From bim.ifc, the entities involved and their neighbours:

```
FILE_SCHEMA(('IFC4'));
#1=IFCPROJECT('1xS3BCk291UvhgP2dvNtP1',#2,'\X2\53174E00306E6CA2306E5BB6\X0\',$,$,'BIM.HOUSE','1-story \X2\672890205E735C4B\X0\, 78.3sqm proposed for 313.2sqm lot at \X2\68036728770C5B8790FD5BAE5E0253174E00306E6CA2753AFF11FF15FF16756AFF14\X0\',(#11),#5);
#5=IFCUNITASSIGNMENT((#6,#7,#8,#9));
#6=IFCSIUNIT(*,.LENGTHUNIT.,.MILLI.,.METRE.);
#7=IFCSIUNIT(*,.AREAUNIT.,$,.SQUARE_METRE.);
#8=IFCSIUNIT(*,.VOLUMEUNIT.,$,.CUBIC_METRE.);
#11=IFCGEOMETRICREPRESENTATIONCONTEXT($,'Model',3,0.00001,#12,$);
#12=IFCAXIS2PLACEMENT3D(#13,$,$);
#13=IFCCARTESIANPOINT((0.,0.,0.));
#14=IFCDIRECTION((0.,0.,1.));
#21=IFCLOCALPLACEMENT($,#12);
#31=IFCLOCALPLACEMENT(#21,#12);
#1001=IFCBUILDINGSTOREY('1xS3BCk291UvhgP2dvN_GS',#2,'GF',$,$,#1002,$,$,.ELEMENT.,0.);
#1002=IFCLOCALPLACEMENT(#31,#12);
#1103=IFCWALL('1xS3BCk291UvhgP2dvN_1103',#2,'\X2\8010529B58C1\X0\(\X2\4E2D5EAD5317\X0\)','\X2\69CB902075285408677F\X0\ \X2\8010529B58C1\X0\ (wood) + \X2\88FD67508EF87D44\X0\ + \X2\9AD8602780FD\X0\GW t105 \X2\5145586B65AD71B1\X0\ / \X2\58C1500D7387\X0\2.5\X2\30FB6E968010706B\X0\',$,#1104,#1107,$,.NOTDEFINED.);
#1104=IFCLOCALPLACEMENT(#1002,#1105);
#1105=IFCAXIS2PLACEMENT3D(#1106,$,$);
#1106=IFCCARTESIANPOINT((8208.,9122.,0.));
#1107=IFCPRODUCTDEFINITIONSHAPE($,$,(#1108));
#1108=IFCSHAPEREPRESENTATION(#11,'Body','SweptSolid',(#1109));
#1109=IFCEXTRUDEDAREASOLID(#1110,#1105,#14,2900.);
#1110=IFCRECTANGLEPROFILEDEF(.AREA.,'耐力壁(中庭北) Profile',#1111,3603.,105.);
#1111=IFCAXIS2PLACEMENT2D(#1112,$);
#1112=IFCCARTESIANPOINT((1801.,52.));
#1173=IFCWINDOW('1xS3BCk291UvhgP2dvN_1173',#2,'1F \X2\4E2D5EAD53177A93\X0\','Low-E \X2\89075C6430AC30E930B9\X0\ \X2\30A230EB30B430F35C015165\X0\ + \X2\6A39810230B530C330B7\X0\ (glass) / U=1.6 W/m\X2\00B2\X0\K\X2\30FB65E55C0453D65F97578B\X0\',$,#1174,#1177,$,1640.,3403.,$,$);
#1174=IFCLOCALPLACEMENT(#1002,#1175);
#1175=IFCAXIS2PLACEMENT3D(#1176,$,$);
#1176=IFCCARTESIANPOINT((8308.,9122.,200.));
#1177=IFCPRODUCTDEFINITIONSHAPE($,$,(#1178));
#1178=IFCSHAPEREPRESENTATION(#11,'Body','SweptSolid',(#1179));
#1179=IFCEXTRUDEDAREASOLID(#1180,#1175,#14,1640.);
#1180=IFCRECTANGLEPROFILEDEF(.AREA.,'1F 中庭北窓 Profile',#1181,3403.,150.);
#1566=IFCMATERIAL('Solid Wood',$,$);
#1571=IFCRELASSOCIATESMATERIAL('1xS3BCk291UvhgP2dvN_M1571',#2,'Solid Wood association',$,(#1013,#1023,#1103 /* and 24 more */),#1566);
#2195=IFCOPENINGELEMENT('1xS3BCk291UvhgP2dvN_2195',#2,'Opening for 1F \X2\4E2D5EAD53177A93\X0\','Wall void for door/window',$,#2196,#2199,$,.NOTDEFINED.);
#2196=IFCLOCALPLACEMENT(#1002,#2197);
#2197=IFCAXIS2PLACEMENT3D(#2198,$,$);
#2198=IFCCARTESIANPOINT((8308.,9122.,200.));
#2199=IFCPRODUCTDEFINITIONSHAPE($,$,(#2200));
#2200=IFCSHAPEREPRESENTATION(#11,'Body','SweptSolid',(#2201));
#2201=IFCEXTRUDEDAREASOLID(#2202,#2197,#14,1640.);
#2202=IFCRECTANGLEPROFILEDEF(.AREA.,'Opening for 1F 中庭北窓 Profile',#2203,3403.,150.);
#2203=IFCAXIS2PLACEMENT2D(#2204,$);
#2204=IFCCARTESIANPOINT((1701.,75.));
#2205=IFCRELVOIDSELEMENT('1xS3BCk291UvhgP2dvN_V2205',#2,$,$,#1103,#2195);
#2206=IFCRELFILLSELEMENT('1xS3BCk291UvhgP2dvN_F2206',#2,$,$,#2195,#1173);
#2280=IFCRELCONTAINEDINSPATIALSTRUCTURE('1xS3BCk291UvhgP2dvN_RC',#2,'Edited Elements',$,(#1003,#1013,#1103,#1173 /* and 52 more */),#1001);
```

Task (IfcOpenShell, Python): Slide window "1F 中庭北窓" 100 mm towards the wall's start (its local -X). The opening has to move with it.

```python
import ifcopenshell
import ifcopenshell.api.geometry
import ifcopenshell.util.placement
import ifcopenshell.util.unit

model = ifcopenshell.open("bim.ifc")
unit_scale = ifcopenshell.util.unit.calculate_unit_scale(model)

window = model.by_id(1173)
opening = window.FillsVoids[0].RelatingOpeningElement
wall = opening.VoidsElements[0].RelatingBuildingElement

wall_matrix = ifcopenshell.util.placement.get_local_placement(wall.ObjectPlacement)
shift = wall_matrix[:3, 0] * -0.1 / unit_scale
before = ifcopenshell.util.placement.get_local_placement(window.ObjectPlacement)[:3, 3].copy()

# The window is not placed relative to its opening, so move both.
for product in (opening, window):
    matrix = ifcopenshell.util.placement.get_local_placement(product.ObjectPlacement)
    matrix[:3, 3] += shift
    ifcopenshell.api.geometry.edit_object_placement(model, product=product, matrix=matrix, is_si=False)

after = ifcopenshell.util.placement.get_local_placement(window.ObjectPlacement)[:3, 3]
print("window moved by", (after - before).round(3) + 0.0)

model.write("bim_v2.ifc")
```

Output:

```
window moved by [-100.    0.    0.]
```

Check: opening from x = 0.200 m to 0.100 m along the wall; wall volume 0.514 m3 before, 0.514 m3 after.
